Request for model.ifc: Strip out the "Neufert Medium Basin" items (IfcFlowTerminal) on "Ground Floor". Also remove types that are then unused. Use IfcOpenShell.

First a look at what the model holds.

```python
import ifcopenshell
import ifcopenshell.util.element

model = ifcopenshell.open("model.ifc")
print(model.schema)
storey = next(s for s in model.by_type("IfcBuildingStorey") if s.Name == "Ground Floor")
terminals = [e for e in ifcopenshell.util.element.get_decomposition(storey) if e.is_a("IfcFlowTerminal")]
seen = {}
for e in terminals:
    element_type = ifcopenshell.util.element.get_type(e)
    name = element_type.Name if element_type not in (None, e) else None
    seen[name] = seen.get(name, 0) + 1
for name, count in sorted(seen.items(), key=str):
    print(count, "x", name)
```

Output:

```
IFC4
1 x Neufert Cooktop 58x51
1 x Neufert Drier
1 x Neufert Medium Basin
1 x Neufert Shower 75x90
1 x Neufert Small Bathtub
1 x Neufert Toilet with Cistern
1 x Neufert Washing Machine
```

```python
import ifcopenshell
import ifcopenshell.api.root
import ifcopenshell.util.element

model = ifcopenshell.open("model.ifc")

storey = next(s for s in model.by_type("IfcBuildingStorey") if s.Name == "Ground Floor")
terminals = [e for e in ifcopenshell.util.element.get_decomposition(storey) if e.is_a("IfcFlowTerminal")]
targets = [e for e in terminals if (t := ifcopenshell.util.element.get_type(e)) not in (None, e) and t.Name == "Neufert Medium Basin"]
types = {ifcopenshell.util.element.get_type(e) for e in targets} - {None, *targets}

for e in targets:
    ifcopenshell.api.root.remove_product(model, product=e)
print(len(targets), "removed")

unused = [t for t in types if not ifcopenshell.util.element.get_types(t)]
for t in unused:
    ifcopenshell.api.root.remove_product(model, product=t)
print(len(unused), "unused types removed")

model.write("model-out.ifc")
```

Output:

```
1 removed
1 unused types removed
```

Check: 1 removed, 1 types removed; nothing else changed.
